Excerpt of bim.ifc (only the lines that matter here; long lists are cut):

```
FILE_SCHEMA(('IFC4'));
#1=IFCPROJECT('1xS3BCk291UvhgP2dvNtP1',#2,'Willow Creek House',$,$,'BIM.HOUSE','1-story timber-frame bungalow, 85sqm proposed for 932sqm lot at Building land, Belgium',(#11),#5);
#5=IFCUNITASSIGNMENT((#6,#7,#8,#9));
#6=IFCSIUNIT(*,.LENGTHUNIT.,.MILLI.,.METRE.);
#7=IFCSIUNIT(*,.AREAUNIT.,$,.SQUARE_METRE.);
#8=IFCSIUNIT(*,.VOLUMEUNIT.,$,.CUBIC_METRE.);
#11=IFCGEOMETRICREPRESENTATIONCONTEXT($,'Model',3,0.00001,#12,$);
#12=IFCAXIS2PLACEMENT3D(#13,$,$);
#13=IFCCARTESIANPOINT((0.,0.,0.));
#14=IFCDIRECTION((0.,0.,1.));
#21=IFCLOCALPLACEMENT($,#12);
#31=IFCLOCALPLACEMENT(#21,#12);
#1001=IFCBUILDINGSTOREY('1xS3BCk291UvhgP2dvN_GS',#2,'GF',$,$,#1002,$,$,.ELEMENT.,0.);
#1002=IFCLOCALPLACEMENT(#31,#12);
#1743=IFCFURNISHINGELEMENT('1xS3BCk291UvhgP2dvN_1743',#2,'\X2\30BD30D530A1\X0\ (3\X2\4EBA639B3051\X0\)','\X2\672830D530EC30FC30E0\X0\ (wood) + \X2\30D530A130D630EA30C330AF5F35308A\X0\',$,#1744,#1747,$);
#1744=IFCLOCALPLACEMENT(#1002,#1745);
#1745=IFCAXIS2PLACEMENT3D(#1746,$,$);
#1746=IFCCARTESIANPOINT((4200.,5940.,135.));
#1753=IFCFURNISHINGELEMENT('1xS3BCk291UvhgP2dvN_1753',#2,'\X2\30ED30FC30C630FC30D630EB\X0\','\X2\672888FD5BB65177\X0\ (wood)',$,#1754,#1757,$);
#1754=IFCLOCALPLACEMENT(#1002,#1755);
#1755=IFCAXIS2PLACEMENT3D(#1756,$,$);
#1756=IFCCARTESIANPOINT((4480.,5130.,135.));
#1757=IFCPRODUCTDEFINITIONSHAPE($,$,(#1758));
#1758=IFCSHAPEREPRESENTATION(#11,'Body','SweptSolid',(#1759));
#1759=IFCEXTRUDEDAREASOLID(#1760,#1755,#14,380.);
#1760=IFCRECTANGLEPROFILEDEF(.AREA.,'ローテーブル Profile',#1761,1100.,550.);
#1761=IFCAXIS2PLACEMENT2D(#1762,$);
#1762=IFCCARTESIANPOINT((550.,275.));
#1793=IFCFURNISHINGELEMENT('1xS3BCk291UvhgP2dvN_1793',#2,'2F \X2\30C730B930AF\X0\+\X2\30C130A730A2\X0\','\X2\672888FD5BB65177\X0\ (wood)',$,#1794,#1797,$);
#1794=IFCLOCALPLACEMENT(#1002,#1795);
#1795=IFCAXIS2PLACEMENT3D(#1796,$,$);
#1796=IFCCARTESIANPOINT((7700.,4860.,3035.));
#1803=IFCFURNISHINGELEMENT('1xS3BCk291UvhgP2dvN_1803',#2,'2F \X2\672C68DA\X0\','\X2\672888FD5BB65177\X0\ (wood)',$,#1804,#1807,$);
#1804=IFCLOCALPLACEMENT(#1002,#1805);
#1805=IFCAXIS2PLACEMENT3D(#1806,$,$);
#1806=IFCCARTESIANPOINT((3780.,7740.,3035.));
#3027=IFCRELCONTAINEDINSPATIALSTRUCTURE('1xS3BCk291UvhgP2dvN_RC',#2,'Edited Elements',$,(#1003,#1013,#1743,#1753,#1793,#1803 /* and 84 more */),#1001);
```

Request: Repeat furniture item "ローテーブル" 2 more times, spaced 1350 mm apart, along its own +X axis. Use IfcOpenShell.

```python
import ifcopenshell
import ifcopenshell.api.geometry
import ifcopenshell.api.root
import ifcopenshell.util.element
import ifcopenshell.util.placement
import ifcopenshell.util.unit

model = ifcopenshell.open("bim.ifc")
unit_scale = ifcopenshell.util.unit.calculate_unit_scale(model)


def reuse_history(source, copy):
    """copy_class also copies each property set's owner history, people and application; keep the originals."""
    for rel in copy.IsDefinedBy:
        if rel.is_a("IfcRelDefinesByProperties") and (history := rel.RelatingPropertyDefinition.OwnerHistory):
            rel.RelatingPropertyDefinition.OwnerHistory = source.OwnerHistory
            ifcopenshell.util.element.remove_deep2(model, history)


source = model.by_guid("1xS3BCk291UvhgP2dvN_1753")
base = ifcopenshell.util.placement.get_local_placement(source.ObjectPlacement)
step = base[:3, 0] * 1.35 / unit_scale

for i in range(1, 3):
    copy = ifcopenshell.api.root.copy_class(model, product=source)
    copy.Representation = ifcopenshell.util.element.copy_deep(
        model, source.Representation, exclude=["IfcGeometricRepresentationContext", "IfcRepresentationMap"]
    )
    reuse_history(source, copy)
    matrix = base.copy()
    matrix[:3, 3] += i * step
    print("added at", matrix[:3, 3].round(3) + 0.0)
    ifcopenshell.api.geometry.edit_object_placement(model, product=copy, matrix=matrix, is_si=False)

model.write("bim_rev.ifc")
```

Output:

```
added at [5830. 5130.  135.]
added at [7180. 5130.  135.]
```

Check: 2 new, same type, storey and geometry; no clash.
